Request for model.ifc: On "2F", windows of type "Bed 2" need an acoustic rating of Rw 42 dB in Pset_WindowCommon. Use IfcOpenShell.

First a look at what the model holds.

```python
import ifcopenshell
import ifcopenshell.util.element

model = ifcopenshell.open("model.ifc")
print(model.schema)
storey = next(s for s in model.by_type("IfcBuildingStorey") if s.Name == "2F")
windows = [e for e in ifcopenshell.util.element.get_decomposition(storey) if e.is_a("IfcWindow")]
seen = {}
for e in windows:
    element_type = ifcopenshell.util.element.get_type(e)
    key = (element_type.Name if element_type != e and element_type else None, ifcopenshell.util.element.get_pset(e, "Pset_WindowCommon", "AcousticRating"))
    seen[key] = seen.get(key, 0) + 1
for (name, value), count in sorted(seen.items(), key=str):
    print(count, "x", name, "|", value)
```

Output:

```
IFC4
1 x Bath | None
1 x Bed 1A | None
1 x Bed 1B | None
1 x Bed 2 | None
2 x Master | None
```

```python
import ifcopenshell
import ifcopenshell.api.pset
import ifcopenshell.util.element

model = ifcopenshell.open("model.ifc")

storey = next(s for s in model.by_type("IfcBuildingStorey") if s.Name == "2F")
windows = [e for e in ifcopenshell.util.element.get_decomposition(storey) if e.is_a("IfcWindow")]

count = 0
for e in windows:
    element_type = ifcopenshell.util.element.get_type(e)
    if element_type in (None, e) or element_type.Name != "Bed 2":
        continue
    # add_pset returns the element's existing set when there is one.
    pset = ifcopenshell.api.pset.add_pset(model, product=e, name="Pset_WindowCommon")
    ifcopenshell.api.pset.edit_pset(model, pset=pset, properties={"AcousticRating": "Rw 42 dB"})
    count += 1

print(count, "windows updated")

model.write("model-out.ifc")
```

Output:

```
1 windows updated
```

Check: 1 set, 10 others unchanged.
